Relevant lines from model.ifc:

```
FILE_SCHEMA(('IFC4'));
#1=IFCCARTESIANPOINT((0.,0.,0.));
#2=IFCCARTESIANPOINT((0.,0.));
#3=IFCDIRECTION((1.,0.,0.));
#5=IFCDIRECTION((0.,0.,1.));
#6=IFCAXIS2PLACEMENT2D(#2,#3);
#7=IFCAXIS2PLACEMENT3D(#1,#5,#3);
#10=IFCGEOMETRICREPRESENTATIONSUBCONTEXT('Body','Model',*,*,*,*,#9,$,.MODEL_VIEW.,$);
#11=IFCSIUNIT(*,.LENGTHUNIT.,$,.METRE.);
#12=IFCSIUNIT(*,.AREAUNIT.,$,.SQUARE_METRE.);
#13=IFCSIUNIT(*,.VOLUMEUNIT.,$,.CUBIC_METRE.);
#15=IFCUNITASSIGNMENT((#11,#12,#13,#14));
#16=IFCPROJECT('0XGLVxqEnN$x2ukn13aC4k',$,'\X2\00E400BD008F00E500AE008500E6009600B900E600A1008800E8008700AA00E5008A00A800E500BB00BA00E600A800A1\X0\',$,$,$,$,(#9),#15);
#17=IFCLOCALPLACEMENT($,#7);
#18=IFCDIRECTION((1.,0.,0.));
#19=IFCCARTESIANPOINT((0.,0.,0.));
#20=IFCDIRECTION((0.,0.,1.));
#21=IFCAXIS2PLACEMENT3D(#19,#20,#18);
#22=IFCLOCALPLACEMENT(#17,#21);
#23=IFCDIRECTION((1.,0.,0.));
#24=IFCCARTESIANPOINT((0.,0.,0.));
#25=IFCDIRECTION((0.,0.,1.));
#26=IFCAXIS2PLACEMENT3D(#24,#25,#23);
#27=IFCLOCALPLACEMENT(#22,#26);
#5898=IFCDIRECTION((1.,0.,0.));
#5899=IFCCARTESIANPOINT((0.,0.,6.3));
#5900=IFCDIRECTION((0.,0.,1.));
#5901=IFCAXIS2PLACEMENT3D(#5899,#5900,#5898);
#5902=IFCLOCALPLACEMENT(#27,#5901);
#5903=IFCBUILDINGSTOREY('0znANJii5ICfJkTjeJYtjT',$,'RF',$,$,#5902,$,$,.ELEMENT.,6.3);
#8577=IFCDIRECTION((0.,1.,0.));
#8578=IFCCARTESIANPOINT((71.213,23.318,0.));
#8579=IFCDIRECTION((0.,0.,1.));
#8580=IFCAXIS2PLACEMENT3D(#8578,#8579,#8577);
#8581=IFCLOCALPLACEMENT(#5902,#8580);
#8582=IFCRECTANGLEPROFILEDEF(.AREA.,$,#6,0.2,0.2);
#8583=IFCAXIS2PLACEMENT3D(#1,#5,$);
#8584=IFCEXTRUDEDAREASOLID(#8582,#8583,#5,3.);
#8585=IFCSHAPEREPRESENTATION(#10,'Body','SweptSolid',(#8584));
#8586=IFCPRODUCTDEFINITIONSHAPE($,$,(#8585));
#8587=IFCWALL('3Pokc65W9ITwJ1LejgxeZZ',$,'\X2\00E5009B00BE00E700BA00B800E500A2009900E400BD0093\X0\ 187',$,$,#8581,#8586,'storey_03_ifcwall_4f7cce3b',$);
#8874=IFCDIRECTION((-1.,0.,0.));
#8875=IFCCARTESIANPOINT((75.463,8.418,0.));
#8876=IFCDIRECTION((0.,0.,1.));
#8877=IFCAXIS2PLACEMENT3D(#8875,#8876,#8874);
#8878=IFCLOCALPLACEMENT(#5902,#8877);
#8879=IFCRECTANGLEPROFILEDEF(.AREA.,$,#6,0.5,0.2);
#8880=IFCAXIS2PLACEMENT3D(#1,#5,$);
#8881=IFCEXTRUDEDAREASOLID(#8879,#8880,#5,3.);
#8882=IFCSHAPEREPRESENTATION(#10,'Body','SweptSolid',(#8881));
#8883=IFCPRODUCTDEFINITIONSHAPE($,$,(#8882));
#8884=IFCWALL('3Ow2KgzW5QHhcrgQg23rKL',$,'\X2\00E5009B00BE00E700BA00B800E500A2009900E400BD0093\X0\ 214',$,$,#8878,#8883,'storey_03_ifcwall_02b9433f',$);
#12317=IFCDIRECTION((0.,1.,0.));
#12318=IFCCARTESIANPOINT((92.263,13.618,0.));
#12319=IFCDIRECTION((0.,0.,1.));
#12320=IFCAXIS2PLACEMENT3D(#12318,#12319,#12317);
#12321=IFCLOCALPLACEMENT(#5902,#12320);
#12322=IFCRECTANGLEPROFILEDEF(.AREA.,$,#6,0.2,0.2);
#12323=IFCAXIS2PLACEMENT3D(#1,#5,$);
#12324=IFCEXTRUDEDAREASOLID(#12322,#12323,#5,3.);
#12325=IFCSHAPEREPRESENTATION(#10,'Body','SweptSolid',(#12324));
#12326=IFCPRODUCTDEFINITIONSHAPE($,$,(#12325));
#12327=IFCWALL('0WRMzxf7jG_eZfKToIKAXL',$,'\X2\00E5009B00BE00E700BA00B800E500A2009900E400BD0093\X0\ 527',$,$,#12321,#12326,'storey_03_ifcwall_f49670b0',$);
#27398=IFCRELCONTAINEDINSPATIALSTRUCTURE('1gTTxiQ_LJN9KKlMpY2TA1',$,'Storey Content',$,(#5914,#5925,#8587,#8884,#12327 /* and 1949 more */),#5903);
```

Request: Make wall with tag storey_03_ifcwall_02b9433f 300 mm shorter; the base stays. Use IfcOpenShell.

```python
import ifcopenshell
import ifcopenshell.geom
import ifcopenshell.util.representation
import ifcopenshell.util.shape
import ifcopenshell.util.unit

model = ifcopenshell.open("model.ifc")
unit_scale = ifcopenshell.util.unit.calculate_unit_scale(model)
settings = ifcopenshell.geom.settings()


def volume(element):
    """Net volume in cubic metres, openings subtracted."""
    shape = ifcopenshell.geom.create_shape(settings, element)
    return ifcopenshell.util.shape.get_volume(shape.geometry)


wall = model.by_guid("3Ow2KgzW5QHhcrgQg23rKL")
before = volume(wall)

body = ifcopenshell.util.representation.get_representation(wall, "Model", "Body")
solid = body.Items[0]
old_height = solid.Depth
solid.Depth -= 0.3 / unit_scale
after = volume(wall)

print(f"height {old_height:g} -> {solid.Depth:g}, volume {before:.3f} -> {after:.3f} m3")

model.write("model_updated.ifc")
```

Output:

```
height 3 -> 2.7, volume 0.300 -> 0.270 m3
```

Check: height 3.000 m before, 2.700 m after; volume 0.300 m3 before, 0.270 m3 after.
